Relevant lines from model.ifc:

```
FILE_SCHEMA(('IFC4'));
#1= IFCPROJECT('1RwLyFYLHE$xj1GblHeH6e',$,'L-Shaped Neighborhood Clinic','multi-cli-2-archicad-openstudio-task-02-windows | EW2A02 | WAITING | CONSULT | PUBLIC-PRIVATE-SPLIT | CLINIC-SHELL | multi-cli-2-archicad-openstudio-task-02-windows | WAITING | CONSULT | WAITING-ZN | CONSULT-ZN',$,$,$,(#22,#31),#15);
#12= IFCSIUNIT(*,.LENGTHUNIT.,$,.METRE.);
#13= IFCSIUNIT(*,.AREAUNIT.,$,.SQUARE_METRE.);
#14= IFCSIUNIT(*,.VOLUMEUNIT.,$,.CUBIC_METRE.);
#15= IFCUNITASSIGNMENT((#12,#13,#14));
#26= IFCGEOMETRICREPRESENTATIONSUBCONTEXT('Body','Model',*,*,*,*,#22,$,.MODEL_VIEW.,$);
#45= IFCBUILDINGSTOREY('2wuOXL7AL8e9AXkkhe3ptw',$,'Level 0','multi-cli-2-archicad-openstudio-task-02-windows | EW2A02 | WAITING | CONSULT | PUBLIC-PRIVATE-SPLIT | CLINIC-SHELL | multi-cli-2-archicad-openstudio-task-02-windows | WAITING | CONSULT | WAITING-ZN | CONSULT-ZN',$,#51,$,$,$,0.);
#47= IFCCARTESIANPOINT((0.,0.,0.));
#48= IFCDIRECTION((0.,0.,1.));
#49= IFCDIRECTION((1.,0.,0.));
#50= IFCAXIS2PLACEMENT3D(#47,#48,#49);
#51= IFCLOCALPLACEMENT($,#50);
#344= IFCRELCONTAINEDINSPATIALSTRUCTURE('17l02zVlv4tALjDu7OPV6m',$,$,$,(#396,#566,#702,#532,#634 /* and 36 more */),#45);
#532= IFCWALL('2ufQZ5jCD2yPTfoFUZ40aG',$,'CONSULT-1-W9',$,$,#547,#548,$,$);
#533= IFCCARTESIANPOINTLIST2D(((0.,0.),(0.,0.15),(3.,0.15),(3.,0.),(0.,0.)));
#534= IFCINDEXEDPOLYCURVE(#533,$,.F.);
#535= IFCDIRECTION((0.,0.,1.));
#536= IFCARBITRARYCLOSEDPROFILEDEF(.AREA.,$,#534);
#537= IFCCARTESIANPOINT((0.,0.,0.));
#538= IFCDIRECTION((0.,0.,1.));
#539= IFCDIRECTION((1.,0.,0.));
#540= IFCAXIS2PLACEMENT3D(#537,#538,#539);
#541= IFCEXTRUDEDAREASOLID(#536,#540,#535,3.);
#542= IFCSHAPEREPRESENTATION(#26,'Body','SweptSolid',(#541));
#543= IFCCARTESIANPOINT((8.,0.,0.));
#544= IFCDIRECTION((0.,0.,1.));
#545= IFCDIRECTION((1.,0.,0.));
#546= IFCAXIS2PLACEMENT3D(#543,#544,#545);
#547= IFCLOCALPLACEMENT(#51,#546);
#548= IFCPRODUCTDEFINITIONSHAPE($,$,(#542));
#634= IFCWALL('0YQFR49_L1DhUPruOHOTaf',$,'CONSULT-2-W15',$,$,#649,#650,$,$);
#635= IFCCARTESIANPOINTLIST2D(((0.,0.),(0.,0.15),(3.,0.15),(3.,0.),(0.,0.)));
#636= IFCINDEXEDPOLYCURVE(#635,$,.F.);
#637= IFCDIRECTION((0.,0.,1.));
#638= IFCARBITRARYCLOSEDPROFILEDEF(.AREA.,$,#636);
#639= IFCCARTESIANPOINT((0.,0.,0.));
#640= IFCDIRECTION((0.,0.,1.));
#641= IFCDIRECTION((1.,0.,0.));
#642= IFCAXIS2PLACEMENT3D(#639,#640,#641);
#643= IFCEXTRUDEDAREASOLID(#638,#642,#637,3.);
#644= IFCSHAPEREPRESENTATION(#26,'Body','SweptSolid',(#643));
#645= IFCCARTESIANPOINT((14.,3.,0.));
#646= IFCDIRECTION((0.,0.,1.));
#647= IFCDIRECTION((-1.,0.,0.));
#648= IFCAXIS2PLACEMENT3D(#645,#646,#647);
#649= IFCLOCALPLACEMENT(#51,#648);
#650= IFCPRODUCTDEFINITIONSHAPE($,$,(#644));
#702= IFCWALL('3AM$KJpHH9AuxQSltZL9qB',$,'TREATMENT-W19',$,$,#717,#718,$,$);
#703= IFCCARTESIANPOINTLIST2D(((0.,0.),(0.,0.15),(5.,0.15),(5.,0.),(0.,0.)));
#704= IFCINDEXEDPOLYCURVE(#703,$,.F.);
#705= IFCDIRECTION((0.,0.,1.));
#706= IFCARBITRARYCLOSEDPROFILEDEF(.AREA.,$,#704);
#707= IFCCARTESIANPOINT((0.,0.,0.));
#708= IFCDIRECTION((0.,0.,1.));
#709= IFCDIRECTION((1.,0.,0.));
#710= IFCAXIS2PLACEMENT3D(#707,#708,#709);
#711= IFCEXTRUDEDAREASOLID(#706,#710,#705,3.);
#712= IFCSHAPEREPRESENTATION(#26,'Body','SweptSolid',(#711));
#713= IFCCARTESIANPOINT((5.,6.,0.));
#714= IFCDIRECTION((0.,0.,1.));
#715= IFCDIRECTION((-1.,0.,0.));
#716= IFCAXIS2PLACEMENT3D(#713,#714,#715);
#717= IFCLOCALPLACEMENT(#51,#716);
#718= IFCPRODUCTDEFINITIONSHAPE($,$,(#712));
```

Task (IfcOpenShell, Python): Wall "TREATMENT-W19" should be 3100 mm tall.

```python
import ifcopenshell
import ifcopenshell.geom
import ifcopenshell.util.representation
import ifcopenshell.util.shape

model = ifcopenshell.open("model.ifc")
settings = ifcopenshell.geom.settings()


def volume(element):
    """Net volume in cubic metres, openings subtracted."""
    shape = ifcopenshell.geom.create_shape(settings, element)
    return ifcopenshell.util.shape.get_volume(shape.geometry)


wall = model.by_id(702)
before = volume(wall)

body = ifcopenshell.util.representation.get_representation(wall, "Model", "Body")
solid = body.Items[0]
old_height = solid.Depth
solid.Depth = 3.1
after = volume(wall)

print(f"height {old_height:g} -> {solid.Depth:g}, volume {before:.3f} -> {after:.3f} m3")

model.write("model_rev.ifc")
```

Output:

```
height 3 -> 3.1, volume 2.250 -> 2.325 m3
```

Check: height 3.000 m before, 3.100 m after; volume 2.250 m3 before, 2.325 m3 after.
